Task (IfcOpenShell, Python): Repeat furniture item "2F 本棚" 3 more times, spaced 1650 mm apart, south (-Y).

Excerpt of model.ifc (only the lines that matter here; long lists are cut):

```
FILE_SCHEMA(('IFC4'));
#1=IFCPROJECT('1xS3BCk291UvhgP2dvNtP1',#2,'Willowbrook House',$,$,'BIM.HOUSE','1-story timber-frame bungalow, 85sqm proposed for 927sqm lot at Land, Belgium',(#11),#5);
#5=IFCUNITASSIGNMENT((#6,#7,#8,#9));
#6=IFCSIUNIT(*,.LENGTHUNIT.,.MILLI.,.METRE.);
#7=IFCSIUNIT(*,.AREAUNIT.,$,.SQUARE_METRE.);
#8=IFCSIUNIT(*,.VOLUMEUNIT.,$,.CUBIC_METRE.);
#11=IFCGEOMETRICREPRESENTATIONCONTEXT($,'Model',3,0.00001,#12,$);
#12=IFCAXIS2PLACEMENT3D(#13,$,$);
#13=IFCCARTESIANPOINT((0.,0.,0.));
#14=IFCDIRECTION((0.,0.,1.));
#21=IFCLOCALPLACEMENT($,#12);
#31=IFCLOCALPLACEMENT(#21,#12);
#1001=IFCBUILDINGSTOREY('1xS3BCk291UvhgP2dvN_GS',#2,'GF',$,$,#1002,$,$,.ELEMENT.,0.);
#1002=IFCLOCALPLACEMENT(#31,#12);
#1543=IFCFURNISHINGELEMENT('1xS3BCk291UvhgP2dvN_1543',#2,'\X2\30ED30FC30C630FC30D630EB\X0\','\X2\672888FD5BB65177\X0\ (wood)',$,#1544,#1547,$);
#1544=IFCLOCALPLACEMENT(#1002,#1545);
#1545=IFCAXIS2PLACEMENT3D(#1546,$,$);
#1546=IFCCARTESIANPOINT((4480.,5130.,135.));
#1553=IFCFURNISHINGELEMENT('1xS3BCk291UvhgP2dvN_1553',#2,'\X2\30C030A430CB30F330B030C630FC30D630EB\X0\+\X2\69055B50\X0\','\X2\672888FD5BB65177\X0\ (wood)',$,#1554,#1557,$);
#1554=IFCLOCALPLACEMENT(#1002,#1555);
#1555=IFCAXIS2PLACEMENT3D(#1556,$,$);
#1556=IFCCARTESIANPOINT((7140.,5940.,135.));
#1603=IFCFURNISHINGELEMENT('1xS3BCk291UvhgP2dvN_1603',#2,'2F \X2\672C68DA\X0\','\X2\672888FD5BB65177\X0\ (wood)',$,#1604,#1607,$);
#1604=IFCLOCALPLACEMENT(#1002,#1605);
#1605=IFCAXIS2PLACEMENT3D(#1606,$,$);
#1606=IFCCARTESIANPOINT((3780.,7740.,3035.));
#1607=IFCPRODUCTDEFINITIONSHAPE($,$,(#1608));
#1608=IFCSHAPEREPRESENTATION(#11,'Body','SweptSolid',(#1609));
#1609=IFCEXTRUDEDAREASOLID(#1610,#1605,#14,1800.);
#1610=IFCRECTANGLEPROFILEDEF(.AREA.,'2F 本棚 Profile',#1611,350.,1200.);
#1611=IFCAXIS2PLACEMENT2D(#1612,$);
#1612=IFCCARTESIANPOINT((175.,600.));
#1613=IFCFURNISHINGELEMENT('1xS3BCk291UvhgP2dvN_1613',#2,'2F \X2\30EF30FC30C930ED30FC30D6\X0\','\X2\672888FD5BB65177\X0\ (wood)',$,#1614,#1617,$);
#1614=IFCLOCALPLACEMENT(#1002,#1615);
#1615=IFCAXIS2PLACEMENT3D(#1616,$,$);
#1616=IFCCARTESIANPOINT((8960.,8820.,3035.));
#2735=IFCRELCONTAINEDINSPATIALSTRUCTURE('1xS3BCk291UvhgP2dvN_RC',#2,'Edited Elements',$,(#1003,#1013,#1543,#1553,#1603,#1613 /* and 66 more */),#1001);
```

```python
import numpy as np
import ifcopenshell
import ifcopenshell.api.geometry
import ifcopenshell.api.root
import ifcopenshell.util.element
import ifcopenshell.util.placement

model = ifcopenshell.open("model.ifc")


def reuse_history(source, copy):
    """copy_class also copies each property set's owner history, people and application; keep the originals."""
    for rel in copy.IsDefinedBy:
        if rel.is_a("IfcRelDefinesByProperties") and (history := rel.RelatingPropertyDefinition.OwnerHistory):
            rel.RelatingPropertyDefinition.OwnerHistory = source.OwnerHistory
            ifcopenshell.util.element.remove_deep2(model, history)


source = model.by_guid("1xS3BCk291UvhgP2dvN_1603")
base = ifcopenshell.util.placement.get_local_placement(source.ObjectPlacement)
step = np.array([0.0, -1.0, 0.0]) * 1650.0

for i in range(1, 4):
    copy = ifcopenshell.api.root.copy_class(model, product=source)
    copy.Representation = ifcopenshell.util.element.copy_deep(
        model, source.Representation, exclude=["IfcGeometricRepresentationContext", "IfcRepresentationMap"]
    )
    reuse_history(source, copy)
    matrix = base.copy()
    matrix[:3, 3] += i * step
    print("added at", matrix[:3, 3].round(3) + 0.0)
    ifcopenshell.api.geometry.edit_object_placement(model, product=copy, matrix=matrix, is_si=False)

model.write("model-out.ifc")
```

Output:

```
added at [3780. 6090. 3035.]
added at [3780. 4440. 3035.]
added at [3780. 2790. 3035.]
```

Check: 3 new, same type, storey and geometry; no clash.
